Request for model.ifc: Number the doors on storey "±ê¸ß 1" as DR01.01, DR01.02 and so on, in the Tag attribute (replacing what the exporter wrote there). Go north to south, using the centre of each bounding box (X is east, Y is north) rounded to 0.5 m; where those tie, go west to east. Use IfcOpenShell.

First a look at what the model holds.

```python
import ifcopenshell
import ifcopenshell.util.element
import ifcopenshell.util.placement

model = ifcopenshell.open("model.ifc")
print(model.schema)
storey = next(s for s in model.by_type("IfcBuildingStorey") if s.Name == "±ê¸ß 1")
doors = [e for e in ifcopenshell.util.element.get_decomposition(storey) if e.is_a("IfcDoor")]
for e in sorted(doors, key=lambda e: e.id()):
    origin = ifcopenshell.util.placement.get_local_placement(e.ObjectPlacement)[:3, 3]
    print(e.id(), e.Tag, e.Name, origin.round(2) + 0.0, sep=" | ")
```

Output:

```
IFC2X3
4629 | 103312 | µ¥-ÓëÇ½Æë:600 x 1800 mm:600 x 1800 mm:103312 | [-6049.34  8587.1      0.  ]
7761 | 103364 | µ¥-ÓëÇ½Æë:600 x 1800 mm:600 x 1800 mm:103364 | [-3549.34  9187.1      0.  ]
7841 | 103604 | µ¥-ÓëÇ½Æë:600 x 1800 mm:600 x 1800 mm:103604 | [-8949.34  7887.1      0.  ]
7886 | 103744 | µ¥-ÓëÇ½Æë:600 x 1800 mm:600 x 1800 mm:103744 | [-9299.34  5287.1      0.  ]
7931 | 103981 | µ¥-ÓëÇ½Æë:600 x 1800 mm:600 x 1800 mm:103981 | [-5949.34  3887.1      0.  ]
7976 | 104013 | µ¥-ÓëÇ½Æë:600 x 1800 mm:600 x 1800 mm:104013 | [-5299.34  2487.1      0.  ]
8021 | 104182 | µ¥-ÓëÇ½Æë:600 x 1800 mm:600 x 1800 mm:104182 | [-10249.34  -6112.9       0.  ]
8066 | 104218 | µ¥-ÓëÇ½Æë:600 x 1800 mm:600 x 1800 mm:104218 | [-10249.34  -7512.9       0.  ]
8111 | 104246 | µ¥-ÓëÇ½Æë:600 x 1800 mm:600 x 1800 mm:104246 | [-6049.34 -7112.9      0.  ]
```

```python
import ifcopenshell
import ifcopenshell.geom
import ifcopenshell.util.element
import ifcopenshell.util.shape

model = ifcopenshell.open("model.ifc")
settings = ifcopenshell.geom.settings()
settings.set("use-world-coords", True)


def centre(element):
    shape = ifcopenshell.geom.create_shape(settings, element)
    return ifcopenshell.util.shape.get_bbox_centroid(shape.geometry)


storey = next(s for s in model.by_type("IfcBuildingStorey") if s.Name == "±ê¸ß 1")
doors = [e for e in ifcopenshell.util.element.get_decomposition(storey) if e.is_a("IfcDoor")]

# Insertion points can sit at a corner or the storey origin, so sort by the geometry (in metres).
centres = {e: centre(e) for e in doors}
doors.sort(key=lambda e: (-round(centres[e][1] / 0.5), centres[e][0]))

for i, e in enumerate(doors, start=1):
    number = f"DR01.{i:02d}"
    e.Tag = number
    print(e.id(), number)

model.write("model-out.ifc")
```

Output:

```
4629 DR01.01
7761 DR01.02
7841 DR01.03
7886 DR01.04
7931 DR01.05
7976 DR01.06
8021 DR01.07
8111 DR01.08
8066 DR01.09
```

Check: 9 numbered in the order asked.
